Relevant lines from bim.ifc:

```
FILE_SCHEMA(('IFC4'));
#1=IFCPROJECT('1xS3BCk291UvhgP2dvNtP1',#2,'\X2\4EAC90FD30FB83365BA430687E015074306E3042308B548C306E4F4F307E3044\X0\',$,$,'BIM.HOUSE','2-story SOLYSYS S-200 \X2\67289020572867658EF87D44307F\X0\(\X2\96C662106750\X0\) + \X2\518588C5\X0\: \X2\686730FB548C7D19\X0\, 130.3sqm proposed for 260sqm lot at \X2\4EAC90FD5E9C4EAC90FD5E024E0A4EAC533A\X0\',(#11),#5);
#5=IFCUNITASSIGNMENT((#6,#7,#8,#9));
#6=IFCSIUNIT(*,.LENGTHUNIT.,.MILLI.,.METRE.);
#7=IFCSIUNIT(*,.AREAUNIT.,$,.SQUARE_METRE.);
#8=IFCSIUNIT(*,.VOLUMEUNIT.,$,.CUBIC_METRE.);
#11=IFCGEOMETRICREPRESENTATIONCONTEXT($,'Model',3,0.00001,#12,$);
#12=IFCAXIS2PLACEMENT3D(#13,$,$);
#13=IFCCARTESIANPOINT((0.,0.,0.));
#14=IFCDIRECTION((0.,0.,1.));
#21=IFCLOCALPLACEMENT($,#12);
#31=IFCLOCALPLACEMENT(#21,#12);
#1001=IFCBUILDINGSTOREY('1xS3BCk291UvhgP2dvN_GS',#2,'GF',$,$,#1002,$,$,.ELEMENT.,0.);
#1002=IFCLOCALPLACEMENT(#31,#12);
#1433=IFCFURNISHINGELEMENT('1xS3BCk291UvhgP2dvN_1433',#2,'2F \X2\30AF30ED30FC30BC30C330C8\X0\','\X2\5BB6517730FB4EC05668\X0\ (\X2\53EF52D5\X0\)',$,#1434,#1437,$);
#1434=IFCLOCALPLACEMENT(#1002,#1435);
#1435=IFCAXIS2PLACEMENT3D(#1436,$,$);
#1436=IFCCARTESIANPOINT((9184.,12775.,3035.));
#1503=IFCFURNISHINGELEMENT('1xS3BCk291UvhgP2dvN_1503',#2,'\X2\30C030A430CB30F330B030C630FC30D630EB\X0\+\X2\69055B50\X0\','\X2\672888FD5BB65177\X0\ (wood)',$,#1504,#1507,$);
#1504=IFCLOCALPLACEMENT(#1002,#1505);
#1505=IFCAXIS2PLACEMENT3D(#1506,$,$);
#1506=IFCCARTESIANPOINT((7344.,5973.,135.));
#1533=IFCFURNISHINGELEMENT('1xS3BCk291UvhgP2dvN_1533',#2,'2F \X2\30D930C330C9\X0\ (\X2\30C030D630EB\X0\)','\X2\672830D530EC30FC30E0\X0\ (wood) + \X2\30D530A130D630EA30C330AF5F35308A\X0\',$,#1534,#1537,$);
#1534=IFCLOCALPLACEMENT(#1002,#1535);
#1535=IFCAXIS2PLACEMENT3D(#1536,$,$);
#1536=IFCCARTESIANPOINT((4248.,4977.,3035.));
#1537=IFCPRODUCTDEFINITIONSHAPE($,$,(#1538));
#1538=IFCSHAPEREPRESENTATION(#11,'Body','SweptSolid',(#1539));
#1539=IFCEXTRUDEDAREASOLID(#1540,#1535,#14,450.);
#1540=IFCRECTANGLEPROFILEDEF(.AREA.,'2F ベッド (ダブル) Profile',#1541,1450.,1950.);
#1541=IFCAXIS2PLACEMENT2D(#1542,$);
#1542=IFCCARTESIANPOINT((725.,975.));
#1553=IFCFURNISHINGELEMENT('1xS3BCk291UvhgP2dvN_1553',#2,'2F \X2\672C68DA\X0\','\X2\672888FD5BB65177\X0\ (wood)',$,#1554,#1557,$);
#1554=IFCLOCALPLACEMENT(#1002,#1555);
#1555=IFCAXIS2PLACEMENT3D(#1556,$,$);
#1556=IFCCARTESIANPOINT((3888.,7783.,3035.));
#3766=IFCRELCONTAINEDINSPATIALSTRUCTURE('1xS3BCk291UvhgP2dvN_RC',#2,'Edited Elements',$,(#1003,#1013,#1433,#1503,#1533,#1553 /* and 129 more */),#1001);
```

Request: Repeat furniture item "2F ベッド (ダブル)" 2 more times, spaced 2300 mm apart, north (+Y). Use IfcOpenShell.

```python
import numpy as np
import ifcopenshell
import ifcopenshell.api.geometry
import ifcopenshell.api.root
import ifcopenshell.util.element
import ifcopenshell.util.placement

model = ifcopenshell.open("bim.ifc")


def reuse_history(source, copy):
    """copy_class also copies each property set's owner history, people and application; keep the originals."""
    for rel in copy.IsDefinedBy:
        if rel.is_a("IfcRelDefinesByProperties") and (history := rel.RelatingPropertyDefinition.OwnerHistory):
            rel.RelatingPropertyDefinition.OwnerHistory = source.OwnerHistory
            ifcopenshell.util.element.remove_deep2(model, history)


source = model.by_guid("1xS3BCk291UvhgP2dvN_1533")
base = ifcopenshell.util.placement.get_local_placement(source.ObjectPlacement)
step = np.array([0.0, 1.0, 0.0]) * 2300.0

for i in range(1, 3):
    copy = ifcopenshell.api.root.copy_class(model, product=source)
    copy.Representation = ifcopenshell.util.element.copy_deep(
        model, source.Representation, exclude=["IfcGeometricRepresentationContext", "IfcRepresentationMap"]
    )
    reuse_history(source, copy)
    matrix = base.copy()
    matrix[:3, 3] += i * step
    print("added at", matrix[:3, 3].round(3) + 0.0)
    ifcopenshell.api.geometry.edit_object_placement(model, product=copy, matrix=matrix, is_si=False)

model.write("bim_rev.ifc")
```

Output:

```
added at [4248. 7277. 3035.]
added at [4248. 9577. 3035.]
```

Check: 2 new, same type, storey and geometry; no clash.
